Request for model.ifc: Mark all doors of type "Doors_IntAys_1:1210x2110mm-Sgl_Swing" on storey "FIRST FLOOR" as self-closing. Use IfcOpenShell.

First a look at what the model holds.

```python
import ifcopenshell
import ifcopenshell.util.element

model = ifcopenshell.open("model.ifc")
print(model.schema)
storey = next(s for s in model.by_type("IfcBuildingStorey") if s.Name == "FIRST FLOOR")
doors = [e for e in ifcopenshell.util.element.get_decomposition(storey) if e.is_a("IfcDoor")]
seen = {}
for e in doors:
    element_type = ifcopenshell.util.element.get_type(e)
    key = (element_type.Name if element_type != e and element_type else None, ifcopenshell.util.element.get_pset(e, "Pset_DoorCommon", "SelfClosing"))
    seen[key] = seen.get(key, 0) + 1
for (name, value), count in sorted(seen.items(), key=str):
    print(count, "x", name, "|", value)
```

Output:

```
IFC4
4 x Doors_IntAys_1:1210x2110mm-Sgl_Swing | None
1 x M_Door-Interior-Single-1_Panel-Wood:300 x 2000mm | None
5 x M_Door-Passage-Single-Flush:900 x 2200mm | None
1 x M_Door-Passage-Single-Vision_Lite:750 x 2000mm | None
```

```python
import ifcopenshell
import ifcopenshell.api.pset
import ifcopenshell.util.element

model = ifcopenshell.open("model.ifc")

storey = next(s for s in model.by_type("IfcBuildingStorey") if s.Name == "FIRST FLOOR")
doors = [e for e in ifcopenshell.util.element.get_decomposition(storey) if e.is_a("IfcDoor")]

count = 0
for e in doors:
    element_type = ifcopenshell.util.element.get_type(e)
    if element_type in (None, e) or element_type.Name != "Doors_IntAys_1:1210x2110mm-Sgl_Swing":
        continue
    # add_pset returns the element's existing set when there is one.
    pset = ifcopenshell.api.pset.add_pset(model, product=e, name="Pset_DoorCommon")
    ifcopenshell.api.pset.edit_pset(model, pset=pset, properties={"SelfClosing": True})
    count += 1

print(count, "doors updated")

model.write("model_v2.ifc")
```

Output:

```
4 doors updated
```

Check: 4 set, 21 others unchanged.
